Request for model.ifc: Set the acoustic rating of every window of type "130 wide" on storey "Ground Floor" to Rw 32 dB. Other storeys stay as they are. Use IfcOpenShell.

First a look at what the model holds.

```python
import ifcopenshell
import ifcopenshell.util.element

model = ifcopenshell.open("model.ifc")
print(model.schema)
storey = next(s for s in model.by_type("IfcBuildingStorey") if s.Name == "Ground Floor")
windows = [e for e in ifcopenshell.util.element.get_decomposition(storey) if e.is_a("IfcWindow")]
seen = {}
for e in windows:
    element_type = ifcopenshell.util.element.get_type(e)
    key = (element_type.Name if element_type != e and element_type else None, ifcopenshell.util.element.get_pset(e, "Pset_WindowCommon", "AcousticRating"))
    seen[key] = seen.get(key, 0) + 1
for (name, value), count in sorted(seen.items(), key=str):
    print(count, "x", name, "|", value)
```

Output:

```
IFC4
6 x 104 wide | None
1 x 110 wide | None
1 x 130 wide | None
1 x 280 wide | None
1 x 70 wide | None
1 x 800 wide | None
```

```python
import ifcopenshell
import ifcopenshell.api.pset
import ifcopenshell.util.element

model = ifcopenshell.open("model.ifc")

storey = next(s for s in model.by_type("IfcBuildingStorey") if s.Name == "Ground Floor")
windows = [e for e in ifcopenshell.util.element.get_decomposition(storey) if e.is_a("IfcWindow")]

count = 0
for e in windows:
    element_type = ifcopenshell.util.element.get_type(e)
    if element_type in (None, e) or element_type.Name != "130 wide":
        continue
    # add_pset returns the element's existing set when there is one.
    pset = ifcopenshell.api.pset.add_pset(model, product=e, name="Pset_WindowCommon")
    ifcopenshell.api.pset.edit_pset(model, pset=pset, properties={"AcousticRating": "Rw 32 dB"})
    count += 1

print(count, "windows updated")

model.write("model_rev.ifc")
```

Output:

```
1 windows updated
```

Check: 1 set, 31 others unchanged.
